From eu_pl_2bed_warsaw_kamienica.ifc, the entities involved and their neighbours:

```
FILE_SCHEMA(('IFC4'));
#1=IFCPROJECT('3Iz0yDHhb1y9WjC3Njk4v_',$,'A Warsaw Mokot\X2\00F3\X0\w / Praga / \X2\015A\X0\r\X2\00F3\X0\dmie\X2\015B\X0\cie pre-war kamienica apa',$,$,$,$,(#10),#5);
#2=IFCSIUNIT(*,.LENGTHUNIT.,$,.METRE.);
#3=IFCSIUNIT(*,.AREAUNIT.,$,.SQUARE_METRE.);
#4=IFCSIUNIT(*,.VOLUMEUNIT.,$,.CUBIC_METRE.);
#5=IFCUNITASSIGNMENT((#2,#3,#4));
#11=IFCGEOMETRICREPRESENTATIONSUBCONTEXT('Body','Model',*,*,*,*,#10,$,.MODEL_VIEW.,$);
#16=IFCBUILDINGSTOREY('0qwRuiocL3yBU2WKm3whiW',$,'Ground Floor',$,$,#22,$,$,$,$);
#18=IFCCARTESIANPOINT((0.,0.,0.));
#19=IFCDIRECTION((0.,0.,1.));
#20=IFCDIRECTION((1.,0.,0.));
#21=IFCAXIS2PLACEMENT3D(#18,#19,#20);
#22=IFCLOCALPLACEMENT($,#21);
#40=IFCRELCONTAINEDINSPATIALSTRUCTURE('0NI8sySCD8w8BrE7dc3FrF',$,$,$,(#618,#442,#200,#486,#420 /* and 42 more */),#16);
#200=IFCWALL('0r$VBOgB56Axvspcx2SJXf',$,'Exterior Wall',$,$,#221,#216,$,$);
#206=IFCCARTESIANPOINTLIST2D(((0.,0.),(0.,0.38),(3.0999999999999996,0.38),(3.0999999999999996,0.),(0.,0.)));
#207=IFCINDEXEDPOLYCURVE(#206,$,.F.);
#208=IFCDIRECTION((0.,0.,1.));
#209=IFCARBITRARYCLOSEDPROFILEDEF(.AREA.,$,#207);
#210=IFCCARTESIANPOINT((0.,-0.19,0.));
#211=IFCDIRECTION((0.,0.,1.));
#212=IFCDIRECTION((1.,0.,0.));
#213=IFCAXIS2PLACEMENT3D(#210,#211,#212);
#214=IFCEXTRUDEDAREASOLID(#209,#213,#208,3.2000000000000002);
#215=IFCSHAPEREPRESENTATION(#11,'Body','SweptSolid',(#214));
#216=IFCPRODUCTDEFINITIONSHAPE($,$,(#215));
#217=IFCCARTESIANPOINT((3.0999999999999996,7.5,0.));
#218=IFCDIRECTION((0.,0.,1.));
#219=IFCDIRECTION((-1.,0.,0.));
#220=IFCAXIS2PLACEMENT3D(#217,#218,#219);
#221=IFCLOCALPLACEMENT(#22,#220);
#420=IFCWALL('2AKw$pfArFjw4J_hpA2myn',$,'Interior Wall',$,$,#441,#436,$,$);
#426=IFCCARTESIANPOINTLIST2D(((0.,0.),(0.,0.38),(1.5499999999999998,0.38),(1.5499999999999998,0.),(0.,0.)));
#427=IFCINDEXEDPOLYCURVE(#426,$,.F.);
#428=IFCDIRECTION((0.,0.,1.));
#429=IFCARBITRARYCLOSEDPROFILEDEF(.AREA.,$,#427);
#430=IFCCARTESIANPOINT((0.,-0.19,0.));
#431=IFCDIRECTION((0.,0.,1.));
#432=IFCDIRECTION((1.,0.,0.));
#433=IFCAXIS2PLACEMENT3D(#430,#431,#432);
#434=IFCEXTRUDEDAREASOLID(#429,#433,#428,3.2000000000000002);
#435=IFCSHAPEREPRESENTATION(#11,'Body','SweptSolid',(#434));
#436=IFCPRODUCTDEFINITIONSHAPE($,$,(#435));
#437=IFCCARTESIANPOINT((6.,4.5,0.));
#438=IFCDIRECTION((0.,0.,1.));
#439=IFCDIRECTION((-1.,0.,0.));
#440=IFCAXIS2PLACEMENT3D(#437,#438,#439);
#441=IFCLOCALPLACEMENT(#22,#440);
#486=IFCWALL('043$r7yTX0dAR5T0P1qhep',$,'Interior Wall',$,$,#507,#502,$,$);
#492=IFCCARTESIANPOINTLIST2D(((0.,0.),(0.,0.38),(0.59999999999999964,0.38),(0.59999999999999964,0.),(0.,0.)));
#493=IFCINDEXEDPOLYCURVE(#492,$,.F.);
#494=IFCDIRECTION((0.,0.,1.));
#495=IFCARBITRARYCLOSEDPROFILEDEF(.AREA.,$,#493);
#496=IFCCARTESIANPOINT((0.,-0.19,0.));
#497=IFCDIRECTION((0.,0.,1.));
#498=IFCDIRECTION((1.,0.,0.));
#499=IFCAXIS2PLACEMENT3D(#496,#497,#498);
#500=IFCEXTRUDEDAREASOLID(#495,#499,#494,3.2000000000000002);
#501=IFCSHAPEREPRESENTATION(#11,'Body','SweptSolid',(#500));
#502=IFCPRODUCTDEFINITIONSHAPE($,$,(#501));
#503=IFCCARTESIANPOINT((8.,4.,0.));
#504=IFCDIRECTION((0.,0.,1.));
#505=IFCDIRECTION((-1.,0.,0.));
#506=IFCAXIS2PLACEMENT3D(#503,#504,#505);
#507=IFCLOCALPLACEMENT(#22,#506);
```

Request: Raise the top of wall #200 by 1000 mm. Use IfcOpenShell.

```python
import ifcopenshell
import ifcopenshell.geom
import ifcopenshell.util.representation
import ifcopenshell.util.shape

model = ifcopenshell.open("eu_pl_2bed_warsaw_kamienica.ifc")
settings = ifcopenshell.geom.settings()


def volume(element):
    """Net volume in cubic metres, openings subtracted."""
    shape = ifcopenshell.geom.create_shape(settings, element)
    return ifcopenshell.util.shape.get_volume(shape.geometry)


wall = model.by_guid("0r$VBOgB56Axvspcx2SJXf")
before = volume(wall)

body = ifcopenshell.util.representation.get_representation(wall, "Model", "Body")
solid = body.Items[0]
old_height = solid.Depth
solid.Depth += 1.0
after = volume(wall)

print(f"height {old_height:g} -> {solid.Depth:g}, volume {before:.3f} -> {after:.3f} m3")

model.write("eu_pl_2bed_warsaw_kamienica_edited.ifc")
```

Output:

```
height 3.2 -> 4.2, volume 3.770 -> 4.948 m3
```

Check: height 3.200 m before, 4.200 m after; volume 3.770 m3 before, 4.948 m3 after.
